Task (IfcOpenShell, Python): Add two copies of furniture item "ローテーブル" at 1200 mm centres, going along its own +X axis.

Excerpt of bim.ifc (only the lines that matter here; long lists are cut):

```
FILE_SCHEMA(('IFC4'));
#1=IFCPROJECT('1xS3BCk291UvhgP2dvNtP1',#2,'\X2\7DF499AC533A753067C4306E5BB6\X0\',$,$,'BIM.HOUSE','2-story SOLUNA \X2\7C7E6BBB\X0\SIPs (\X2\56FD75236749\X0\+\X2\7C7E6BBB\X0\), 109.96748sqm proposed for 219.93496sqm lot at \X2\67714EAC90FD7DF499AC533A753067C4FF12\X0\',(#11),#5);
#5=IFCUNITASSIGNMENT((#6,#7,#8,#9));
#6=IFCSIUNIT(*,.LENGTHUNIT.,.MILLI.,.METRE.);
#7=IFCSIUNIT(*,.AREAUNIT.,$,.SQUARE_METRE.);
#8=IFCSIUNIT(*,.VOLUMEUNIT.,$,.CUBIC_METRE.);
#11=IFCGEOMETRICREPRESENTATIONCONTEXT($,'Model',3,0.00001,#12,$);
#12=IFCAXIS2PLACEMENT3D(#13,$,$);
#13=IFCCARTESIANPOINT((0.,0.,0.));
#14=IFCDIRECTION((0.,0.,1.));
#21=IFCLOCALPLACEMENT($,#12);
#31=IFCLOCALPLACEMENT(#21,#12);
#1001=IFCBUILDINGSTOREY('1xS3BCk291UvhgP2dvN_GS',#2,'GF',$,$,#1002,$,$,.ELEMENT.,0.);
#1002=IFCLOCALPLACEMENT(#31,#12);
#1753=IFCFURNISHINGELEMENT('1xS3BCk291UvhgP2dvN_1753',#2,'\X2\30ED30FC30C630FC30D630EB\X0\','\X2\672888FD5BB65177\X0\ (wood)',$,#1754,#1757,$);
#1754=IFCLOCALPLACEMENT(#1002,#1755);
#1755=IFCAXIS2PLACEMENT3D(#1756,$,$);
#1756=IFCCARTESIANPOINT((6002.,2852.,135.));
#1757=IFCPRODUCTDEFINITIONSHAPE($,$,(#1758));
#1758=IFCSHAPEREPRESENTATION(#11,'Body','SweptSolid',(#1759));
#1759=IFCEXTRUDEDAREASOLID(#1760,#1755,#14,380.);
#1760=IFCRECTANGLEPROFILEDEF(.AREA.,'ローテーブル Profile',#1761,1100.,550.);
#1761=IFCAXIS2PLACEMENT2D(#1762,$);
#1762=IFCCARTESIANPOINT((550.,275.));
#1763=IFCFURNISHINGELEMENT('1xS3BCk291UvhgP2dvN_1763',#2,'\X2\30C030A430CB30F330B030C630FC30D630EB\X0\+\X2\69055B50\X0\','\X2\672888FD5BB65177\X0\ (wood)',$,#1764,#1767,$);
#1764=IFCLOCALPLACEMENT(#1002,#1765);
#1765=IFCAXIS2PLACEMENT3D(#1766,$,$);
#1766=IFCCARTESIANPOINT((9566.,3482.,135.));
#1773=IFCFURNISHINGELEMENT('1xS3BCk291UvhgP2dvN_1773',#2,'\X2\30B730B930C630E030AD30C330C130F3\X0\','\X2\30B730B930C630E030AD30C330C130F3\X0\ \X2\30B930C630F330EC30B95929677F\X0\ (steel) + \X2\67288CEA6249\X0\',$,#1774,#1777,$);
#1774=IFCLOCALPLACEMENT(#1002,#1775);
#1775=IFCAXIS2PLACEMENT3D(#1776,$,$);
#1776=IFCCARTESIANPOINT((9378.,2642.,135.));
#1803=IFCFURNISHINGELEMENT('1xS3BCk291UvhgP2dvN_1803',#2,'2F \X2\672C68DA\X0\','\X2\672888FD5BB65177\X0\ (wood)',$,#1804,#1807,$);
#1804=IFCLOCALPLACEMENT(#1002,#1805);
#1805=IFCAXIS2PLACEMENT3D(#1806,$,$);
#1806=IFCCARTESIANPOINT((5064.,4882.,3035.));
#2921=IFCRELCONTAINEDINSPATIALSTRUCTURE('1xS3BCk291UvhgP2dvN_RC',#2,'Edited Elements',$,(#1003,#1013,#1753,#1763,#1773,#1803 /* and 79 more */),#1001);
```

```python
import ifcopenshell
import ifcopenshell.api.geometry
import ifcopenshell.api.root
import ifcopenshell.util.element
import ifcopenshell.util.placement
import ifcopenshell.util.unit

model = ifcopenshell.open("bim.ifc")
unit_scale = ifcopenshell.util.unit.calculate_unit_scale(model)


def reuse_history(source, copy):
    """copy_class also copies each property set's owner history, people and application; keep the originals."""
    for rel in copy.IsDefinedBy:
        if rel.is_a("IfcRelDefinesByProperties") and (history := rel.RelatingPropertyDefinition.OwnerHistory):
            rel.RelatingPropertyDefinition.OwnerHistory = source.OwnerHistory
            ifcopenshell.util.element.remove_deep2(model, history)


source = model.by_guid("1xS3BCk291UvhgP2dvN_1753")
base = ifcopenshell.util.placement.get_local_placement(source.ObjectPlacement)
step = base[:3, 0] * 1.2 / unit_scale

for i in range(1, 3):
    copy = ifcopenshell.api.root.copy_class(model, product=source)
    copy.Representation = ifcopenshell.util.element.copy_deep(
        model, source.Representation, exclude=["IfcGeometricRepresentationContext", "IfcRepresentationMap"]
    )
    reuse_history(source, copy)
    matrix = base.copy()
    matrix[:3, 3] += i * step
    print("added at", matrix[:3, 3].round(3) + 0.0)
    ifcopenshell.api.geometry.edit_object_placement(model, product=copy, matrix=matrix, is_si=False)

model.write("bim_rev.ifc")
```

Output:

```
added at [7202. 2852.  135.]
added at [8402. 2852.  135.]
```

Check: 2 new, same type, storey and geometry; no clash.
